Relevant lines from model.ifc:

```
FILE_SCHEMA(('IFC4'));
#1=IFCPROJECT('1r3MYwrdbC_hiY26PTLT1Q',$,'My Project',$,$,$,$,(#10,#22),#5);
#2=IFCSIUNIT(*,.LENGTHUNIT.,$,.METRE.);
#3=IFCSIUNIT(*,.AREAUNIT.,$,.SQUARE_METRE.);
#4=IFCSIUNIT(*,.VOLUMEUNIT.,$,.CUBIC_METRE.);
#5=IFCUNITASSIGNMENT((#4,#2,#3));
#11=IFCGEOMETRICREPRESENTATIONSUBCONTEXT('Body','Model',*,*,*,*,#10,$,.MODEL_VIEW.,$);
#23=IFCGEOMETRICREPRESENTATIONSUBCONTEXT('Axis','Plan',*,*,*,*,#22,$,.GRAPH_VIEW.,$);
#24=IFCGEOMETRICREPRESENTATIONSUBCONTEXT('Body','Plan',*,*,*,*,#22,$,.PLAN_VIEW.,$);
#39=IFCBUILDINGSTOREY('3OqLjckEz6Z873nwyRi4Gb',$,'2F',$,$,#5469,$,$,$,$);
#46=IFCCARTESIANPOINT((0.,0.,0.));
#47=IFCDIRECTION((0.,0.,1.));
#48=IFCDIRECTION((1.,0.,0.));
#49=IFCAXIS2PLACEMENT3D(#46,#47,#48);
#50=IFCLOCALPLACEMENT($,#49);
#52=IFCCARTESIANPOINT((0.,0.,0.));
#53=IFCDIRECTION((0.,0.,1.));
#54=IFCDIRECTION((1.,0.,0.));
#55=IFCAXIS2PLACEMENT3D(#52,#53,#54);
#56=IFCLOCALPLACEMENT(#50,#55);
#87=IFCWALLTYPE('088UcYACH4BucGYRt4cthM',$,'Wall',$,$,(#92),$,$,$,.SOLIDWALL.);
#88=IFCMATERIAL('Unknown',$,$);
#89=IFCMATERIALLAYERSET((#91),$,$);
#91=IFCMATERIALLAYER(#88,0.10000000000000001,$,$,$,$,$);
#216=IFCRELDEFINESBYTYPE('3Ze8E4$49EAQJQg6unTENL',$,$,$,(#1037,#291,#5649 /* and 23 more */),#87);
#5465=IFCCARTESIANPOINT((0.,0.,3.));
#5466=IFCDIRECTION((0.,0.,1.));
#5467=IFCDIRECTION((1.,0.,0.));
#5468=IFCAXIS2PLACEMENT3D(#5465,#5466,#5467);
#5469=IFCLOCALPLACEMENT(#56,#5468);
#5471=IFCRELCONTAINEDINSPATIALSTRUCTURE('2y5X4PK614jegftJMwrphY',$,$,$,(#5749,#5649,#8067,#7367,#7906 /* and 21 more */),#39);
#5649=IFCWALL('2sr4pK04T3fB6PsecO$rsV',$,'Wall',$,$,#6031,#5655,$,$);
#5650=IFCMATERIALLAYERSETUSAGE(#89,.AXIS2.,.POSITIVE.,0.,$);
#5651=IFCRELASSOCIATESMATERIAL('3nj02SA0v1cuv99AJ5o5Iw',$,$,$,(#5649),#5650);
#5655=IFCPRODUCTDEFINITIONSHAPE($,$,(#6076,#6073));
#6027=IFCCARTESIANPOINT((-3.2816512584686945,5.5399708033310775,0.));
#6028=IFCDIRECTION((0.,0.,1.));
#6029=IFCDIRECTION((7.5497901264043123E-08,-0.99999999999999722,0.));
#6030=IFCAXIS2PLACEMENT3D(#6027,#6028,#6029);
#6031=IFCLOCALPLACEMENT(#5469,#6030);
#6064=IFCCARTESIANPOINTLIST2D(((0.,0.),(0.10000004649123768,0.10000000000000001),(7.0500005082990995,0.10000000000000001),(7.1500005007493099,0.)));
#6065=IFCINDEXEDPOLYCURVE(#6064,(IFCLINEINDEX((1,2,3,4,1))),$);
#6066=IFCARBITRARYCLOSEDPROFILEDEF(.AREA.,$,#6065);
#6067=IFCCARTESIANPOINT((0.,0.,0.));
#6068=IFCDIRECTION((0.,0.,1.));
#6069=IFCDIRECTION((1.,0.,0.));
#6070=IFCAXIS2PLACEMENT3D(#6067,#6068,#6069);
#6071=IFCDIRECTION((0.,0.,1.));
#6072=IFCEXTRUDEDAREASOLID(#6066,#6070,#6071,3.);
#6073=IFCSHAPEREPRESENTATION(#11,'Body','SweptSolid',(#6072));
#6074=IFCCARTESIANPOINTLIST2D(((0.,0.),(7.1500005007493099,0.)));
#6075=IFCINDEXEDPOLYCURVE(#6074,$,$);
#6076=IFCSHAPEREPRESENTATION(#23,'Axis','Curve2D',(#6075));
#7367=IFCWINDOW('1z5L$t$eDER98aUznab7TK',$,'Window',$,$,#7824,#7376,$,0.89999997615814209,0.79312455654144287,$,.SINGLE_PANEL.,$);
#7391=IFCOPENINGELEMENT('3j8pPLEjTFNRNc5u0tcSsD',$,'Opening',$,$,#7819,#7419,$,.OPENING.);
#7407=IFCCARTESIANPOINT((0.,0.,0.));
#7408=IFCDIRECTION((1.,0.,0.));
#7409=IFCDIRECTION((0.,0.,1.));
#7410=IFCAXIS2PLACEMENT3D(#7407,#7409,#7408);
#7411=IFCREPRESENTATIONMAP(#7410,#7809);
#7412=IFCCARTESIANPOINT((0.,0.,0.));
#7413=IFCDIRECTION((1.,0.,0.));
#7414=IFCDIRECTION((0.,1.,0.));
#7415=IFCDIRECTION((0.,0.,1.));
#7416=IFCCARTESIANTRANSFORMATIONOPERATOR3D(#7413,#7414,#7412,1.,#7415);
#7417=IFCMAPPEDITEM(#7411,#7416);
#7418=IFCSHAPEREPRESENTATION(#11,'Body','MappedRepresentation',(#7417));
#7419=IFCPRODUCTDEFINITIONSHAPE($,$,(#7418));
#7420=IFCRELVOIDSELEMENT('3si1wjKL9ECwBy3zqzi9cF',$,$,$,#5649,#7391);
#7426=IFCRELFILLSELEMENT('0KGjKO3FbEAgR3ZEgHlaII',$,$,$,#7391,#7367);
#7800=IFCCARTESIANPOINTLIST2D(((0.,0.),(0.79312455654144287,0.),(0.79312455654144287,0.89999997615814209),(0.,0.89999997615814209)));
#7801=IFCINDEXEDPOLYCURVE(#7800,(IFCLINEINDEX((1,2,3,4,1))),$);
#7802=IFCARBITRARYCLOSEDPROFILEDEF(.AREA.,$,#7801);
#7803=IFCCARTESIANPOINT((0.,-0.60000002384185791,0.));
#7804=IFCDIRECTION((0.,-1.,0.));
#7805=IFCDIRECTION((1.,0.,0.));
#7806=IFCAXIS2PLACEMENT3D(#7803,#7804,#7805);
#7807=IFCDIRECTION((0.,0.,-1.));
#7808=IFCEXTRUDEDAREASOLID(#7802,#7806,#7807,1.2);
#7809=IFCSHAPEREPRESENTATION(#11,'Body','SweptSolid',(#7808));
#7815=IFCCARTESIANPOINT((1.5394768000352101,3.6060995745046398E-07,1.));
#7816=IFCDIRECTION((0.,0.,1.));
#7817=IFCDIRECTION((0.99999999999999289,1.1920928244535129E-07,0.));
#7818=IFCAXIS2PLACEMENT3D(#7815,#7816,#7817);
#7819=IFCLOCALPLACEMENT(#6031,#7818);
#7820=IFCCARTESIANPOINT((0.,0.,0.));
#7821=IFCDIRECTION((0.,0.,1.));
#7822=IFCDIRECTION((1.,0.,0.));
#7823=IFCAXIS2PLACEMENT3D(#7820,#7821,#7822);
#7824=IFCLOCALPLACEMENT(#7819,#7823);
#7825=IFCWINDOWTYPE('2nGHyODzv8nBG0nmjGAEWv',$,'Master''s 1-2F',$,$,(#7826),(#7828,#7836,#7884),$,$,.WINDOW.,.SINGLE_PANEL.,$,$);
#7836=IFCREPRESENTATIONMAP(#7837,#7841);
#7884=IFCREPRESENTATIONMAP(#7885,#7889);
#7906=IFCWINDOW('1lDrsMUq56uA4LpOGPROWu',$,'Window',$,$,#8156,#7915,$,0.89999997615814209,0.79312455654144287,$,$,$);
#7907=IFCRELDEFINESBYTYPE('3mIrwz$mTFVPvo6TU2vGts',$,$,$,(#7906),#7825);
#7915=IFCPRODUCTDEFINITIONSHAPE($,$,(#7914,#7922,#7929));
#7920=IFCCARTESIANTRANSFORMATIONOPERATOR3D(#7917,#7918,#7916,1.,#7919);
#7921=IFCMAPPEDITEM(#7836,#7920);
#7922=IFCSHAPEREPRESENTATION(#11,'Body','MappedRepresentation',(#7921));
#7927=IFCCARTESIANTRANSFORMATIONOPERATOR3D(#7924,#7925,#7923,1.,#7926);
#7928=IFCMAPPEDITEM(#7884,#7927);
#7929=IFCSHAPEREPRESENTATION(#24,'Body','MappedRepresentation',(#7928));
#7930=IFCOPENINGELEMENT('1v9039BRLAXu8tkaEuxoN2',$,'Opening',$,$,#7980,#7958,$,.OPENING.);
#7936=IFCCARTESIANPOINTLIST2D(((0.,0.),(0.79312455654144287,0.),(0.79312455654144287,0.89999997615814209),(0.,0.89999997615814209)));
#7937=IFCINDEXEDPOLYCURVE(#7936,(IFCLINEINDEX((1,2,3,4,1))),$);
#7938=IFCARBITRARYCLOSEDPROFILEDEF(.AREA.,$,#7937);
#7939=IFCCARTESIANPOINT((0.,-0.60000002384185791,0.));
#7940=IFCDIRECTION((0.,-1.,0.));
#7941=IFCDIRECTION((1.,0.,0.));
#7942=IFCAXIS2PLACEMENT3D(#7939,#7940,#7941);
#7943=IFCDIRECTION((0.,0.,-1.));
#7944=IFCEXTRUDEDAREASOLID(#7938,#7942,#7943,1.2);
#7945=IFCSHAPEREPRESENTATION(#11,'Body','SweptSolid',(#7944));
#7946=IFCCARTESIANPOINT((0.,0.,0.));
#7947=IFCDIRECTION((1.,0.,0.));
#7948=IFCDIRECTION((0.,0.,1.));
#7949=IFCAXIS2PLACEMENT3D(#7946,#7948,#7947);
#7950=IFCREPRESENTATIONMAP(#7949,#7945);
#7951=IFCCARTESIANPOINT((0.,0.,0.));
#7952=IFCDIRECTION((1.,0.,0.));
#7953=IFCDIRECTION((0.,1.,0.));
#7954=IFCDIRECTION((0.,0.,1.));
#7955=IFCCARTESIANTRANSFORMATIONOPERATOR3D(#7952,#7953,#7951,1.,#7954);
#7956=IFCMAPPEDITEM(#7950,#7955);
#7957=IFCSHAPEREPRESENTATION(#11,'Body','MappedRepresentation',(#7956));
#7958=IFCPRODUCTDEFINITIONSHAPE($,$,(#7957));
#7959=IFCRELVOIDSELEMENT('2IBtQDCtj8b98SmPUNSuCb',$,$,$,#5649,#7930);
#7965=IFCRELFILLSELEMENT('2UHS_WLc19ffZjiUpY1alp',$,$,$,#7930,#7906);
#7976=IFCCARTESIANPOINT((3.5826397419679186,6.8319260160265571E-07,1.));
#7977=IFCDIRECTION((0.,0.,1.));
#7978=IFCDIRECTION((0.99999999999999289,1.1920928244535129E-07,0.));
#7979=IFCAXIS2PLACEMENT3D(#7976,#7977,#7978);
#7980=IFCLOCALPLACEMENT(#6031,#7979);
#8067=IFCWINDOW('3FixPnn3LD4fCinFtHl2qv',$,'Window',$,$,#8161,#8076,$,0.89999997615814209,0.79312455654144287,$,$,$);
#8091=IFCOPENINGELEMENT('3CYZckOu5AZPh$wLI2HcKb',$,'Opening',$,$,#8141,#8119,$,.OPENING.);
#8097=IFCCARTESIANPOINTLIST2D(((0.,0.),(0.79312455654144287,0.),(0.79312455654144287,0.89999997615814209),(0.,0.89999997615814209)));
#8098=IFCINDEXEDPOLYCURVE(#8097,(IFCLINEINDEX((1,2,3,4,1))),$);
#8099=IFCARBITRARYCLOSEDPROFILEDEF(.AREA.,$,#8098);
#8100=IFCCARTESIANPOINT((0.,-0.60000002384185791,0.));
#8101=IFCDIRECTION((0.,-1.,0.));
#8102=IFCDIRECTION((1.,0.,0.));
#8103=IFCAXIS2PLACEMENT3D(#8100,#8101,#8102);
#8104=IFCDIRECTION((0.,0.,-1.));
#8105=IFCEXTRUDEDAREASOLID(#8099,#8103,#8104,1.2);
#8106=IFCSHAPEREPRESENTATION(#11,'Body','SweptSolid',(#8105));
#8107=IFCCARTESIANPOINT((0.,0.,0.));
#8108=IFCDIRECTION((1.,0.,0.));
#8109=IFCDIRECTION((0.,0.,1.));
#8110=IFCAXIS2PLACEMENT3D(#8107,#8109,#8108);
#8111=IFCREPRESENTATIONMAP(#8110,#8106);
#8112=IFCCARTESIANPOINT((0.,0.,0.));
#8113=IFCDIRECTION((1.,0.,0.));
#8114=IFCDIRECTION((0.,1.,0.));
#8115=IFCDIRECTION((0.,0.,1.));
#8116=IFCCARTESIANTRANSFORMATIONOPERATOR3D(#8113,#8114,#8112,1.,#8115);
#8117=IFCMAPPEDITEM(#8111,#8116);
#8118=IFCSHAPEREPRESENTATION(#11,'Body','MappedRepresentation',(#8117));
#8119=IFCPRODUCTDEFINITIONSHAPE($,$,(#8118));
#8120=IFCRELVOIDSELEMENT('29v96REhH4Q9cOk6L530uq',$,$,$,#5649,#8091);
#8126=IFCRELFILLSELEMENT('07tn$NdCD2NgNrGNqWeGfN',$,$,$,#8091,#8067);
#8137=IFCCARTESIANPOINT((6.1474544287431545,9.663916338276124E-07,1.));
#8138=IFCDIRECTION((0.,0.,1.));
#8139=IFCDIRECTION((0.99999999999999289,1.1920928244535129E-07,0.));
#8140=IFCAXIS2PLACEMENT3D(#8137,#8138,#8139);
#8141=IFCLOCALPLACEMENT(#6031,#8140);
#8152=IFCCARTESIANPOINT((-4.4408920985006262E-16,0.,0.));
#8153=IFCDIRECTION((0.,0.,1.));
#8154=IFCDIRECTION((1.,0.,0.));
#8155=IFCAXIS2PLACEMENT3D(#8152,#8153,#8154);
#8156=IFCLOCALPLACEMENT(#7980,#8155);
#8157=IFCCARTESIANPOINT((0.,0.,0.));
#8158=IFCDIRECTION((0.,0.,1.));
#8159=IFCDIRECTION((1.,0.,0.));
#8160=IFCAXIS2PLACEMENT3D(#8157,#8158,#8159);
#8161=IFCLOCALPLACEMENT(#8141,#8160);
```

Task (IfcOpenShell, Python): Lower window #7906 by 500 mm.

```python
import numpy as np
import ifcopenshell
import ifcopenshell.api.geometry
import ifcopenshell.util.placement
import ifcopenshell.util.unit

model = ifcopenshell.open("model.ifc")
unit_scale = ifcopenshell.util.unit.calculate_unit_scale(model)

window = model.by_guid("1lDrsMUq56uA4LpOGPROWu")
opening = window.FillsVoids[0].RelatingOpeningElement
dz = -0.5

shift = np.array([0.0, 0.0, dz])
# The window is placed relative to its opening, so it follows when the opening moves.
matrix = ifcopenshell.util.placement.get_local_placement(opening.ObjectPlacement)
matrix[:3, 3] += shift
ifcopenshell.api.geometry.edit_object_placement(
    model, product=opening, matrix=matrix, is_si=False, should_transform_children=True
)

print(f"moved by {dz * unit_scale:+.3f} m")

model.write("model-out.ifc")
```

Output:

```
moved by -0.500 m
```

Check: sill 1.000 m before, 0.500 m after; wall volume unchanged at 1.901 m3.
